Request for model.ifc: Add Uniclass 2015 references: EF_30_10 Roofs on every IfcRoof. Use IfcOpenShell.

First a look at what the model holds.

```python
import ifcopenshell

model = ifcopenshell.open("model.ifc")
print(model.schema)
print("classifications:", [c.Name for c in model.by_type("IfcClassification")])
for ifc_class in ("IfcDoor", "IfcRoof", "IfcStair", "IfcWall", "IfcWindow"):
    print(ifc_class, len(model.by_type(ifc_class)))
```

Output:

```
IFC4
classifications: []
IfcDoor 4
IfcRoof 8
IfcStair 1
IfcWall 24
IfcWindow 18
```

```python
import ifcopenshell
import ifcopenshell.api.classification

model = ifcopenshell.open("model.ifc")

system = ifcopenshell.api.classification.add_classification(model, classification="Uniclass 2015")

codes = {
    "IfcRoof": ("EF_30_10", "Roofs"),
}
for ifc_class, (code, name) in codes.items():
    products = model.by_type(ifc_class)
    ifcopenshell.api.classification.add_reference(
        model, products=products, classification=system, identification=code, name=name
    )
    print(code, len(products))

model.write("model_rev.ifc")
```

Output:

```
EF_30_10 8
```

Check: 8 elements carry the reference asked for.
